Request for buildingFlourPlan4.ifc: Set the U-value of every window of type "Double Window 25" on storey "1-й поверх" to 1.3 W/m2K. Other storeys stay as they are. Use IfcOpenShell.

First a look at what the model holds.

```python
import ifcopenshell
import ifcopenshell.util.element

model = ifcopenshell.open("buildingFlourPlan4.ifc")
print(model.schema)
storey = next(s for s in model.by_type("IfcBuildingStorey") if s.Name == "1-й поверх")
windows = [e for e in ifcopenshell.util.element.get_decomposition(storey) if e.is_a("IfcWindow")]
seen = {}
for e in windows:
    element_type = ifcopenshell.util.element.get_type(e)
    key = (element_type.Name if element_type != e and element_type else None, ifcopenshell.util.element.get_pset(e, "Pset_WindowCommon", "ThermalTransmittance"))
    seen[key] = seen.get(key, 0) + 1
for (name, value), count in sorted(seen.items(), key=str):
    print(count, "x", name, "|", value)
```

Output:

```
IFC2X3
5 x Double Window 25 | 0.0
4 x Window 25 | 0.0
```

```python
import ifcopenshell
import ifcopenshell.api.pset
import ifcopenshell.util.element

model = ifcopenshell.open("buildingFlourPlan4.ifc")

storey = next(s for s in model.by_type("IfcBuildingStorey") if s.Name == "1-й поверх")
windows = [e for e in ifcopenshell.util.element.get_decomposition(storey) if e.is_a("IfcWindow")]

count = 0
for e in windows:
    element_type = ifcopenshell.util.element.get_type(e)
    if element_type in (None, e) or element_type.Name != "Double Window 25":
        continue
    # add_pset returns the element's existing set when there is one.
    pset = ifcopenshell.api.pset.add_pset(model, product=e, name="Pset_WindowCommon")
    ifcopenshell.api.pset.edit_pset(model, pset=pset, properties={"ThermalTransmittance": 1.3})
    count += 1

print(count, "windows updated")

model.write("buildingFlourPlan4_edited.ifc")
```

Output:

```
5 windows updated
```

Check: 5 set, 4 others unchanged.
